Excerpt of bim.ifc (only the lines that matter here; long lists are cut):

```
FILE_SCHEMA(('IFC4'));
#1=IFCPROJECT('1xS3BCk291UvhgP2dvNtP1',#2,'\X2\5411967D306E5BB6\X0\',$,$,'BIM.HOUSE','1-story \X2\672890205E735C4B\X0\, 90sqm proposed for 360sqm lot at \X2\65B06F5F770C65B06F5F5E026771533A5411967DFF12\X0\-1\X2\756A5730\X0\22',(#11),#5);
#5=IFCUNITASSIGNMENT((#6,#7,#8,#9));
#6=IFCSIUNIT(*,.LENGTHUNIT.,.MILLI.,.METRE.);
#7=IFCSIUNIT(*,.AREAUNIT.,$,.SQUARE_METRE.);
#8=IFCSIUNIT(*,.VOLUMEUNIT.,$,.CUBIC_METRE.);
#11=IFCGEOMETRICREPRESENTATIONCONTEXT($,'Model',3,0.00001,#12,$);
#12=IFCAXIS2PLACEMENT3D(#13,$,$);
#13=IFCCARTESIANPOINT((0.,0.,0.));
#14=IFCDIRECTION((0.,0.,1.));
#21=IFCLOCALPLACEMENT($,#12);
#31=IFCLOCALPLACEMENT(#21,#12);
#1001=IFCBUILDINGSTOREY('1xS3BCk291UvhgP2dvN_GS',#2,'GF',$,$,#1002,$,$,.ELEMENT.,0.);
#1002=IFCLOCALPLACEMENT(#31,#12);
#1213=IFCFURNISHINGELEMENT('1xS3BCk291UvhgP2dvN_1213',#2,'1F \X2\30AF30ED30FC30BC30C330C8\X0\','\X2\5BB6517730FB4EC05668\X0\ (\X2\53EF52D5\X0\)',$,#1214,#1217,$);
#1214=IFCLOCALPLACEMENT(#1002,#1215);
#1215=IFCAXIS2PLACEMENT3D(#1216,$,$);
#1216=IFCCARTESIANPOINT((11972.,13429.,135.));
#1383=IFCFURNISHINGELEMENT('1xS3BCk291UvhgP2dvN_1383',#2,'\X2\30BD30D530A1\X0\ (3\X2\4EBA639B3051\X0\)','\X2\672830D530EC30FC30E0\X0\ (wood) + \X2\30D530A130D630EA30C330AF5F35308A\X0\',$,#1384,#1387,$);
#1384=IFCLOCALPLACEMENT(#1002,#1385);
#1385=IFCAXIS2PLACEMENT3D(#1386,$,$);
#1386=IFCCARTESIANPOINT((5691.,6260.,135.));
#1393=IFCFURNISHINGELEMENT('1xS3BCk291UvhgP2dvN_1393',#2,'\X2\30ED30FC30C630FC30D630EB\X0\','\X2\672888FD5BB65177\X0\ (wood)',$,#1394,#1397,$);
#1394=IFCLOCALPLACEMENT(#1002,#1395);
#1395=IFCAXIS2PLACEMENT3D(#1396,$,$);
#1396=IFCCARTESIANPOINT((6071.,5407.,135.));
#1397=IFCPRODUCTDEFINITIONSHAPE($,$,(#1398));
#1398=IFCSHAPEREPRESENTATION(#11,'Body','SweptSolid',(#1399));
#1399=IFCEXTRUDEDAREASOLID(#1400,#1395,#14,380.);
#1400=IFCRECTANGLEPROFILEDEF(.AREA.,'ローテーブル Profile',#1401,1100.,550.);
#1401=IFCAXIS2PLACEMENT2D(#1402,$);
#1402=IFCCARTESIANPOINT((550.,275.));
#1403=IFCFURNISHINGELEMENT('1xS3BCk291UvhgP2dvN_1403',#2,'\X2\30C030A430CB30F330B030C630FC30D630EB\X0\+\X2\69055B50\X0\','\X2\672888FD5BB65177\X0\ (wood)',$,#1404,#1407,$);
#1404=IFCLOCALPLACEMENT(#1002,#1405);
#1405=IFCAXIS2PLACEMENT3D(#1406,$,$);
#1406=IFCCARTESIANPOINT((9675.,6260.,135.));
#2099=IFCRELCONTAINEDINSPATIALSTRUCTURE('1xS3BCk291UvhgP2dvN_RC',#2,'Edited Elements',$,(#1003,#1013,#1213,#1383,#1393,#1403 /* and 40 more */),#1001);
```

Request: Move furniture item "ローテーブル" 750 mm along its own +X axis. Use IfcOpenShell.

```python
import ifcopenshell
import ifcopenshell.api.geometry
import ifcopenshell.util.placement
import ifcopenshell.util.unit

model = ifcopenshell.open("bim.ifc")
unit_scale = ifcopenshell.util.unit.calculate_unit_scale(model)

item = model.by_id(1393)
matrix = ifcopenshell.util.placement.get_local_placement(item.ObjectPlacement)
matrix[:3, 3] += matrix[:3, 0] * 0.75 / unit_scale
ifcopenshell.api.geometry.edit_object_placement(model, product=item, matrix=matrix, is_si=False)

print(ifcopenshell.util.placement.get_local_placement(item.ObjectPlacement).round(3) + 0.0)

model.write("bim_rev.ifc")
```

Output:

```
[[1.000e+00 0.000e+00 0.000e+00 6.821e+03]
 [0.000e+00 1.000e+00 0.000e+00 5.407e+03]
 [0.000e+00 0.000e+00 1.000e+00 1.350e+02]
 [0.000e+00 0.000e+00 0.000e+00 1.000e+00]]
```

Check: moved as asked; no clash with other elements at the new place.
